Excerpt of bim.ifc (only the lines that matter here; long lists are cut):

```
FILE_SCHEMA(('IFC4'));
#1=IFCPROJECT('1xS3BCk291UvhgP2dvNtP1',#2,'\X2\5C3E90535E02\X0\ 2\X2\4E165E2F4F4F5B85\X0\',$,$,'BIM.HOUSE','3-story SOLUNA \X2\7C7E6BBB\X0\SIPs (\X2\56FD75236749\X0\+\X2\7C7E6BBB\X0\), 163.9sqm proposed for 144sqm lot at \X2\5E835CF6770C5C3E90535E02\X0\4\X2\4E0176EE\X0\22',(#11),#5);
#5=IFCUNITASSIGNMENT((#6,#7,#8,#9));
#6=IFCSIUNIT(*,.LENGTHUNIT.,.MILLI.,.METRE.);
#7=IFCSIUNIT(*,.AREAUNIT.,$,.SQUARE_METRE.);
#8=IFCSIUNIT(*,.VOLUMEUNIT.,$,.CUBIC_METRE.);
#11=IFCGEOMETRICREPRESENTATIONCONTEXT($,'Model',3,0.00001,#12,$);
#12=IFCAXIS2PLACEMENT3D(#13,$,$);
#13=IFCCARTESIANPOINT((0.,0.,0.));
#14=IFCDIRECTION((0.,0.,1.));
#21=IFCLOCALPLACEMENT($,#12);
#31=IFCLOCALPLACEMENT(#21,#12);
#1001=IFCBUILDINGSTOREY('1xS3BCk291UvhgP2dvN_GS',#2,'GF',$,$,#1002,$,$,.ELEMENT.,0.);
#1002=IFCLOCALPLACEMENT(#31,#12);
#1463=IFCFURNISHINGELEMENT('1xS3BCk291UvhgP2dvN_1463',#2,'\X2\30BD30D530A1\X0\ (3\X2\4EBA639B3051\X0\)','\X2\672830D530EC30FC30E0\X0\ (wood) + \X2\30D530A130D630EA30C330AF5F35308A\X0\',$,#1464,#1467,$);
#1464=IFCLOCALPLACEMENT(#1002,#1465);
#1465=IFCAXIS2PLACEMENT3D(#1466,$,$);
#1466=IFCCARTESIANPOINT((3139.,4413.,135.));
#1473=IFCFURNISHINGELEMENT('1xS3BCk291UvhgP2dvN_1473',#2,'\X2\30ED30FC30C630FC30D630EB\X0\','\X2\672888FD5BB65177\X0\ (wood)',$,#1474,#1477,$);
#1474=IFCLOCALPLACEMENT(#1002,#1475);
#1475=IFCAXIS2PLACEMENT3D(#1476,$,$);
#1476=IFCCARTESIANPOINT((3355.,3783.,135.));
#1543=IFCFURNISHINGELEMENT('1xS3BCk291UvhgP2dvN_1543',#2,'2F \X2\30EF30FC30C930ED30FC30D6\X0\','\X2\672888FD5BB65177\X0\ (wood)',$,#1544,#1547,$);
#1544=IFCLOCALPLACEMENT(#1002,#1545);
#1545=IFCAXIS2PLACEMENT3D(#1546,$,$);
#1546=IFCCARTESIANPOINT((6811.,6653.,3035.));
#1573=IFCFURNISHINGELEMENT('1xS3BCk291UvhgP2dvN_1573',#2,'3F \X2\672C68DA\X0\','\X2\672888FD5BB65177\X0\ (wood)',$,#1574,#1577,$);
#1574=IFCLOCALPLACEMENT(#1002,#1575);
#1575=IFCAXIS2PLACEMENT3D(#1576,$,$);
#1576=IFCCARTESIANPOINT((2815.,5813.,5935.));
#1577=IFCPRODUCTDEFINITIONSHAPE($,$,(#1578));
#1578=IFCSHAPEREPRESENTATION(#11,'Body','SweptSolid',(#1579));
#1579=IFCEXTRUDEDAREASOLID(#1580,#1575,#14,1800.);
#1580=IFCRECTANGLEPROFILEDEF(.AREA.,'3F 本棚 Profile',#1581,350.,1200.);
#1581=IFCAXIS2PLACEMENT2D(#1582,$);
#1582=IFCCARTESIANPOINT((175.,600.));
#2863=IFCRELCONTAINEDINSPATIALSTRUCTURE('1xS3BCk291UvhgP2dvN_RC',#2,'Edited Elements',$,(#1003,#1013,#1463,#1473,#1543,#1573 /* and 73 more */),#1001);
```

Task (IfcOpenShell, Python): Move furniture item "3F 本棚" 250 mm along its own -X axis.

```python
import ifcopenshell
import ifcopenshell.api.geometry
import ifcopenshell.util.placement
import ifcopenshell.util.unit

model = ifcopenshell.open("bim.ifc")
unit_scale = ifcopenshell.util.unit.calculate_unit_scale(model)

item = model.by_guid("1xS3BCk291UvhgP2dvN_1573")
matrix = ifcopenshell.util.placement.get_local_placement(item.ObjectPlacement)
matrix[:3, 3] -= matrix[:3, 0] * 0.25 / unit_scale
ifcopenshell.api.geometry.edit_object_placement(model, product=item, matrix=matrix, is_si=False)

print(ifcopenshell.util.placement.get_local_placement(item.ObjectPlacement).round(3) + 0.0)

model.write("bim_rev.ifc")
```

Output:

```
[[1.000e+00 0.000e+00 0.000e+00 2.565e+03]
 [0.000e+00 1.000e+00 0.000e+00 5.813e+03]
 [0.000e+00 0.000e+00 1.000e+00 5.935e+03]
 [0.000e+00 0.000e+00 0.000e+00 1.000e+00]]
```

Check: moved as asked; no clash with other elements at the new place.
